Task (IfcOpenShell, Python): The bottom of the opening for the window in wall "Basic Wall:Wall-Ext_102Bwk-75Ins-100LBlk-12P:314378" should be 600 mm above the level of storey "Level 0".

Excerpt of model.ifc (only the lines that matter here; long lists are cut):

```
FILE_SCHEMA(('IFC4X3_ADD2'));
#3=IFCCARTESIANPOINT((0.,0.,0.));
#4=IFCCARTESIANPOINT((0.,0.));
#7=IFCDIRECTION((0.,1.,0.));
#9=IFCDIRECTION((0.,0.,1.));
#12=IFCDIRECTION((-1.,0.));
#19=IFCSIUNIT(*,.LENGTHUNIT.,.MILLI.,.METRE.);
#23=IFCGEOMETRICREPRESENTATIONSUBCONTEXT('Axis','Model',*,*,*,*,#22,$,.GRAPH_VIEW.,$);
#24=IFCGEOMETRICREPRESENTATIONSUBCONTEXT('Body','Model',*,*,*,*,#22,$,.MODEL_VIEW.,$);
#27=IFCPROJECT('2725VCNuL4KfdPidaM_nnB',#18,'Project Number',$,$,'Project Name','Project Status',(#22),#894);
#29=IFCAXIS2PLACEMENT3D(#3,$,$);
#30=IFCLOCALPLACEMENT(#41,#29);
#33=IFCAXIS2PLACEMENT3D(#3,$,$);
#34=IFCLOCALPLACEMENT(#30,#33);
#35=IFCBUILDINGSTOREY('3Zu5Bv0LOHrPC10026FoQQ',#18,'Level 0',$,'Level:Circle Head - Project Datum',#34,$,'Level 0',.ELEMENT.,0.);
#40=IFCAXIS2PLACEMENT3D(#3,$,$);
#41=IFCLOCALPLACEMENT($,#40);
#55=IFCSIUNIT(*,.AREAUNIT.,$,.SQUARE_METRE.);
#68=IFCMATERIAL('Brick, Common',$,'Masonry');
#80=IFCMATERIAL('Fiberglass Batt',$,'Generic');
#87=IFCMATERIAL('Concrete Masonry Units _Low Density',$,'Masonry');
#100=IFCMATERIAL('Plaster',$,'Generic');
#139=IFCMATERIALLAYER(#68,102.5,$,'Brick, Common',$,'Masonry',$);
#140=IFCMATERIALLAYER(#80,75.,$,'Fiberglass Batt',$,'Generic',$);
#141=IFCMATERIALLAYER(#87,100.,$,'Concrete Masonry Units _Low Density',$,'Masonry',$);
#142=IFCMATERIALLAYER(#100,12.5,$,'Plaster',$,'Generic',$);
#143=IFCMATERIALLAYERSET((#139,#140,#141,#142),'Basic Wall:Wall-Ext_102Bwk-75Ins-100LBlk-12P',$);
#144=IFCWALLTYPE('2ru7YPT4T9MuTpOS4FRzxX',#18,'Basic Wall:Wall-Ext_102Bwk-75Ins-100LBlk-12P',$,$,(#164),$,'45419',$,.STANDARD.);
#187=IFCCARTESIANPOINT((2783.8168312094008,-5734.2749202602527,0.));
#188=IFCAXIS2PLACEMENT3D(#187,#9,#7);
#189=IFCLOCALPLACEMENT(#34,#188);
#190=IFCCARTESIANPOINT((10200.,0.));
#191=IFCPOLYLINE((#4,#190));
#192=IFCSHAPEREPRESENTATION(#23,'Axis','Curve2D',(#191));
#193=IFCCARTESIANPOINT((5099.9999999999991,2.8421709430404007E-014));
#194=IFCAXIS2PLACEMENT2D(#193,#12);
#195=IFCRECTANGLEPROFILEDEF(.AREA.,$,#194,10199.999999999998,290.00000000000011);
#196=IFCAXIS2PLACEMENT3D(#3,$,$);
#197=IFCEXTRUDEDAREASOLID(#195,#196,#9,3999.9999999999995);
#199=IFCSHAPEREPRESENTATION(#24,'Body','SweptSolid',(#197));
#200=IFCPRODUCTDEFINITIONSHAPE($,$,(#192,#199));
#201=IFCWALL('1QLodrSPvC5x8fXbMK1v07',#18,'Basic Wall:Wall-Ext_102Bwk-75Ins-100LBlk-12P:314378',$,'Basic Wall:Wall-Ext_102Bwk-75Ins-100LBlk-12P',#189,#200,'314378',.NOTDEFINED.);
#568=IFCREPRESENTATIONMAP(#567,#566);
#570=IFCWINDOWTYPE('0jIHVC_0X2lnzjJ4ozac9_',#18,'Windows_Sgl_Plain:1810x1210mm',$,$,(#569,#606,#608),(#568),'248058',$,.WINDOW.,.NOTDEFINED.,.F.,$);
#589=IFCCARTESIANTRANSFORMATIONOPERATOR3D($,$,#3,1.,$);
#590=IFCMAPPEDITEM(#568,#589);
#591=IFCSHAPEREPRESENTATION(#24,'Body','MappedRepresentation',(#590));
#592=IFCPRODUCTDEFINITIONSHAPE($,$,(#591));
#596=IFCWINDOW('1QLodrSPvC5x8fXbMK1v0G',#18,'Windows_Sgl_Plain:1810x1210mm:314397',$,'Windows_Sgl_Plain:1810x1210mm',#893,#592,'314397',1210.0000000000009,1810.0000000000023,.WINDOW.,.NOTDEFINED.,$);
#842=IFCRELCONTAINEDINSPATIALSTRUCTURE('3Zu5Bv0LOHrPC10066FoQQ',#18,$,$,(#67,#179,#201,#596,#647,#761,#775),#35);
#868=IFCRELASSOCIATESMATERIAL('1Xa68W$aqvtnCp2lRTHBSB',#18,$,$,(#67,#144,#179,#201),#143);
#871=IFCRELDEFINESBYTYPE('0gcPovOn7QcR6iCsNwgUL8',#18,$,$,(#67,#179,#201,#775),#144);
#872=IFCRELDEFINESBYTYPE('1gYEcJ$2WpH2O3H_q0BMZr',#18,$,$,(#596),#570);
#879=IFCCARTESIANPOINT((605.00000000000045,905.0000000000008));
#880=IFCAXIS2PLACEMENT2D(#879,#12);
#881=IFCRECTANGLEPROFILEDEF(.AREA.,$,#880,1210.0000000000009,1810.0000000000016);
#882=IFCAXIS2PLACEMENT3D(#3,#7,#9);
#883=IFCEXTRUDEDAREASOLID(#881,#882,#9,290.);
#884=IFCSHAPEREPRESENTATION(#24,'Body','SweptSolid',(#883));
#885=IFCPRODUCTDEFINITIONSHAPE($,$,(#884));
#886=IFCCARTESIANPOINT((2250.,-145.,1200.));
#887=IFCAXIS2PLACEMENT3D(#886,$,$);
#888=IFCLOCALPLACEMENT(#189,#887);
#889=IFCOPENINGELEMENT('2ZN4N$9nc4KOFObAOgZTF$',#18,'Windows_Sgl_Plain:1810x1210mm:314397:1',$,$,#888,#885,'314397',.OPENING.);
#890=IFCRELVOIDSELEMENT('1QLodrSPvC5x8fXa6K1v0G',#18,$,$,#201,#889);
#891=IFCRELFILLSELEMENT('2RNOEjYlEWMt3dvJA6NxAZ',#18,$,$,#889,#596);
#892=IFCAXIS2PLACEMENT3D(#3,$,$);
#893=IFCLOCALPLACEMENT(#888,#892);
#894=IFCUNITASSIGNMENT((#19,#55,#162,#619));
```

```python
import numpy as np
import ifcopenshell
import ifcopenshell.api.geometry
import ifcopenshell.geom
import ifcopenshell.util.element
import ifcopenshell.util.placement
import ifcopenshell.util.shape
import ifcopenshell.util.unit

model = ifcopenshell.open("model.ifc")
unit_scale = ifcopenshell.util.unit.calculate_unit_scale(model)

window = model.by_guid("1QLodrSPvC5x8fXbMK1v0G")
opening = window.FillsVoids[0].RelatingOpeningElement
storey = ifcopenshell.util.element.get_container(window, ifc_class="IfcBuildingStorey")
level = ifcopenshell.util.placement.get_local_placement(storey.ObjectPlacement)[2, 3]

# The opening's origin need not be at the sill, so measure its lowest point.
shape = ifcopenshell.geom.create_shape(ifcopenshell.geom.settings(), opening)
bottom = ifcopenshell.util.shape.get_shape_bottom_elevation(shape, shape.geometry) / unit_scale
dz = level + 600.0 - bottom

shift = np.array([0.0, 0.0, dz])
# The window is placed relative to its opening, so it follows when the opening moves.
matrix = ifcopenshell.util.placement.get_local_placement(opening.ObjectPlacement)
matrix[:3, 3] += shift
ifcopenshell.api.geometry.edit_object_placement(
    model, product=opening, matrix=matrix, is_si=False, should_transform_children=True
)

print(f"moved by {dz * unit_scale:+.3f} m")

model.write("model-out.ifc")
```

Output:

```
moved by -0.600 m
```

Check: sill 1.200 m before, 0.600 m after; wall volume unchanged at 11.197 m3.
